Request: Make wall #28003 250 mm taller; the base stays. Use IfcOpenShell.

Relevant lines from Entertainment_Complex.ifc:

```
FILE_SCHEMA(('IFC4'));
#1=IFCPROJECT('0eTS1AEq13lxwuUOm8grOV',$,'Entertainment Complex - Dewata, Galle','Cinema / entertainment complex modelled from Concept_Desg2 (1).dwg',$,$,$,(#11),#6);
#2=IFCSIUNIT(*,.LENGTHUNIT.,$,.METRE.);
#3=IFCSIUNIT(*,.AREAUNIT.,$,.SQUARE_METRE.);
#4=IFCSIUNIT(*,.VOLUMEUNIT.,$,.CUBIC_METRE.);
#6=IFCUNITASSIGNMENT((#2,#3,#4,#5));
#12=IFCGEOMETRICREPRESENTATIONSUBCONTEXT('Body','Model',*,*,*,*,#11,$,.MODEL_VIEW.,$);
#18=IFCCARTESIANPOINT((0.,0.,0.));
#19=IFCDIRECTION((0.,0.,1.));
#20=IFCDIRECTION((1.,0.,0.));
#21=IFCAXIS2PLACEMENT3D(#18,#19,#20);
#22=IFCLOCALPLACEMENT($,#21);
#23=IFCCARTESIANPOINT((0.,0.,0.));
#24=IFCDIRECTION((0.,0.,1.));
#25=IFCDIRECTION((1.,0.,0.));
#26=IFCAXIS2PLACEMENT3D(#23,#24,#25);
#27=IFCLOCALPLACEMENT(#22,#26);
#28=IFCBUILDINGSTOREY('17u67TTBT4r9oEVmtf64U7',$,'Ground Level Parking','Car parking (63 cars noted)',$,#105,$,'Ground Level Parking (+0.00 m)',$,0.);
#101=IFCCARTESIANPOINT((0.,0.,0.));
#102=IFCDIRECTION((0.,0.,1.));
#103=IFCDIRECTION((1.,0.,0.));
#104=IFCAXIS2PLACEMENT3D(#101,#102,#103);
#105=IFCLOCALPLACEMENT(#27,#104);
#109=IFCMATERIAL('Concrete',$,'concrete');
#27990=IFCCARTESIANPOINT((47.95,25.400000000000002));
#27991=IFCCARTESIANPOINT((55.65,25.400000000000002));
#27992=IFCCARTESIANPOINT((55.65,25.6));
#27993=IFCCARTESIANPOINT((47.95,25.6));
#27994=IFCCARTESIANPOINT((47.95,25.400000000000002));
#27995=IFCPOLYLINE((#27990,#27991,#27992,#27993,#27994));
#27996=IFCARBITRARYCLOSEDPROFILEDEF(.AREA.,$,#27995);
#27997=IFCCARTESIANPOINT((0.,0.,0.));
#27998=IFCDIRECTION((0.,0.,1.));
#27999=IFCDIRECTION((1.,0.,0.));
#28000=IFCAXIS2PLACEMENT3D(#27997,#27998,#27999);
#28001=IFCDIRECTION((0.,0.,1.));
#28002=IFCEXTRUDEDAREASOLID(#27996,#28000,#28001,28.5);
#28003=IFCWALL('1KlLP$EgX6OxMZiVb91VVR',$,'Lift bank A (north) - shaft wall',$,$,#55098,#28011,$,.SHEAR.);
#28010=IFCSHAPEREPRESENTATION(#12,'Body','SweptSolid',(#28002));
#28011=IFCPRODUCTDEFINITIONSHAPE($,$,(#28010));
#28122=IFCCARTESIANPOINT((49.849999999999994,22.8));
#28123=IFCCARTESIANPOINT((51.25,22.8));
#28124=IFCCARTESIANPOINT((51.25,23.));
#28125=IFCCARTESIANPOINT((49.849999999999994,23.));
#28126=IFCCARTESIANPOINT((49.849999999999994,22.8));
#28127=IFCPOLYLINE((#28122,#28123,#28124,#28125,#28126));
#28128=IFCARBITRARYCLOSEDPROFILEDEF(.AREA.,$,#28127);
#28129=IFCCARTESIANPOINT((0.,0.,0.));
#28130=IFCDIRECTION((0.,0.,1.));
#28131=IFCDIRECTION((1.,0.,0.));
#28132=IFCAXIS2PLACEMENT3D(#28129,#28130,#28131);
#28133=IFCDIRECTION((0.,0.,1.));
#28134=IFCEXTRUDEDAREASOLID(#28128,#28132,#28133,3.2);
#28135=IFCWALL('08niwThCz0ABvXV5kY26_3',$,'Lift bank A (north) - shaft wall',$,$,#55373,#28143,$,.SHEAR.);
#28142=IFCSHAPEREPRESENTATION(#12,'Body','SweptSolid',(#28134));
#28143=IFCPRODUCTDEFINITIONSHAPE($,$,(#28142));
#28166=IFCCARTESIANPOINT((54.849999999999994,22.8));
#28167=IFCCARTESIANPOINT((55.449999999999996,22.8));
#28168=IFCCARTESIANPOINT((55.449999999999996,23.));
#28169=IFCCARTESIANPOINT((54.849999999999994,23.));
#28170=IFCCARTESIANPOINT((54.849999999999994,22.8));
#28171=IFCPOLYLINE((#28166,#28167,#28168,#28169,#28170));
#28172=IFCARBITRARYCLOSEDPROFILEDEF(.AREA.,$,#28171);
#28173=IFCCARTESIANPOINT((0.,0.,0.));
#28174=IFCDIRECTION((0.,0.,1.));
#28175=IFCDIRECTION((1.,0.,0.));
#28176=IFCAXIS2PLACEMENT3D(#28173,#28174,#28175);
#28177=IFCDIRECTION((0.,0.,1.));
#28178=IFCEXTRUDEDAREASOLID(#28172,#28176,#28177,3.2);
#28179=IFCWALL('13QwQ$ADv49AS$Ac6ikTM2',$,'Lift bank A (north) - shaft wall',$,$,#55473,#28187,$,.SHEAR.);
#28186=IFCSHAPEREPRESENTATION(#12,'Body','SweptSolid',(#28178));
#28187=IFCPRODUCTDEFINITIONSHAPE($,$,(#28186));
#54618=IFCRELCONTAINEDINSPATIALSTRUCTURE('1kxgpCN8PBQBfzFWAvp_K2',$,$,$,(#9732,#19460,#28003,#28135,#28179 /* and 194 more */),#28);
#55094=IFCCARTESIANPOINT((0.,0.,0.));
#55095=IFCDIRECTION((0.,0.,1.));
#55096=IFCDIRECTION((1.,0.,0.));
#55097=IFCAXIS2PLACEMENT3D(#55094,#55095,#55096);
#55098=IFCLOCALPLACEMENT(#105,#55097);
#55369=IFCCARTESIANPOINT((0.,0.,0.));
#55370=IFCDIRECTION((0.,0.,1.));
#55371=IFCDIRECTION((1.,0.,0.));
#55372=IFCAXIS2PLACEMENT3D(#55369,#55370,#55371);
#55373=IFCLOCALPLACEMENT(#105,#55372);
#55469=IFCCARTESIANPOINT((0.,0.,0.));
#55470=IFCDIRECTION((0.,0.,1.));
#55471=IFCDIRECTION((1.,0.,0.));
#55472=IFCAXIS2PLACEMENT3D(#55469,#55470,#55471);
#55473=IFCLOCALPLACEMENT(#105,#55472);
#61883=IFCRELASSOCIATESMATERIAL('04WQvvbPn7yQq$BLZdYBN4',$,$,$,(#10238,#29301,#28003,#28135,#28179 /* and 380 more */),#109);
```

```python
import ifcopenshell
import ifcopenshell.geom
import ifcopenshell.util.representation
import ifcopenshell.util.shape

model = ifcopenshell.open("Entertainment_Complex.ifc")
settings = ifcopenshell.geom.settings()


def volume(element):
    """Net volume in cubic metres, openings subtracted."""
    shape = ifcopenshell.geom.create_shape(settings, element)
    return ifcopenshell.util.shape.get_volume(shape.geometry)


wall = model.by_guid("1KlLP$EgX6OxMZiVb91VVR")
before = volume(wall)

body = ifcopenshell.util.representation.get_representation(wall, "Model", "Body")
solid = body.Items[0]
old_height = solid.Depth
solid.Depth += 0.25
after = volume(wall)

print(f"height {old_height:g} -> {solid.Depth:g}, volume {before:.3f} -> {after:.3f} m3")

model.write("Entertainment_Complex_v2.ifc")
```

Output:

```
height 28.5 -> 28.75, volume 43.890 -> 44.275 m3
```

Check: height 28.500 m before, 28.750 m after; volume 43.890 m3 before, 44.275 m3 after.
